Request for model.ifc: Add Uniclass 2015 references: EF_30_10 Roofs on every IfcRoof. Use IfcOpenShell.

First a look at what the model holds.

```python
import ifcopenshell

model = ifcopenshell.open("model.ifc")
print(model.schema)
print("classifications:", [c.Name for c in model.by_type("IfcClassification")])
for ifc_class in ("IfcDoor", "IfcRoof", "IfcStair", "IfcWall", "IfcWindow"):
    print(ifc_class, len(model.by_type(ifc_class)))
```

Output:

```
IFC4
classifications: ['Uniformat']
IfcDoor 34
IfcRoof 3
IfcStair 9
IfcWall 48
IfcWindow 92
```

```python
import ifcopenshell
import ifcopenshell.api.classification

model = ifcopenshell.open("model.ifc")

system = ifcopenshell.api.classification.add_classification(model, classification="Uniclass 2015")

codes = {
    "IfcRoof": ("EF_30_10", "Roofs"),
}
for ifc_class, (code, name) in codes.items():
    products = model.by_type(ifc_class)
    ifcopenshell.api.classification.add_reference(
        model, products=products, classification=system, identification=code, name=name
    )
    print(code, len(products))

model.write("model_rev.ifc")
```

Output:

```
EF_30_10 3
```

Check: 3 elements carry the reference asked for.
